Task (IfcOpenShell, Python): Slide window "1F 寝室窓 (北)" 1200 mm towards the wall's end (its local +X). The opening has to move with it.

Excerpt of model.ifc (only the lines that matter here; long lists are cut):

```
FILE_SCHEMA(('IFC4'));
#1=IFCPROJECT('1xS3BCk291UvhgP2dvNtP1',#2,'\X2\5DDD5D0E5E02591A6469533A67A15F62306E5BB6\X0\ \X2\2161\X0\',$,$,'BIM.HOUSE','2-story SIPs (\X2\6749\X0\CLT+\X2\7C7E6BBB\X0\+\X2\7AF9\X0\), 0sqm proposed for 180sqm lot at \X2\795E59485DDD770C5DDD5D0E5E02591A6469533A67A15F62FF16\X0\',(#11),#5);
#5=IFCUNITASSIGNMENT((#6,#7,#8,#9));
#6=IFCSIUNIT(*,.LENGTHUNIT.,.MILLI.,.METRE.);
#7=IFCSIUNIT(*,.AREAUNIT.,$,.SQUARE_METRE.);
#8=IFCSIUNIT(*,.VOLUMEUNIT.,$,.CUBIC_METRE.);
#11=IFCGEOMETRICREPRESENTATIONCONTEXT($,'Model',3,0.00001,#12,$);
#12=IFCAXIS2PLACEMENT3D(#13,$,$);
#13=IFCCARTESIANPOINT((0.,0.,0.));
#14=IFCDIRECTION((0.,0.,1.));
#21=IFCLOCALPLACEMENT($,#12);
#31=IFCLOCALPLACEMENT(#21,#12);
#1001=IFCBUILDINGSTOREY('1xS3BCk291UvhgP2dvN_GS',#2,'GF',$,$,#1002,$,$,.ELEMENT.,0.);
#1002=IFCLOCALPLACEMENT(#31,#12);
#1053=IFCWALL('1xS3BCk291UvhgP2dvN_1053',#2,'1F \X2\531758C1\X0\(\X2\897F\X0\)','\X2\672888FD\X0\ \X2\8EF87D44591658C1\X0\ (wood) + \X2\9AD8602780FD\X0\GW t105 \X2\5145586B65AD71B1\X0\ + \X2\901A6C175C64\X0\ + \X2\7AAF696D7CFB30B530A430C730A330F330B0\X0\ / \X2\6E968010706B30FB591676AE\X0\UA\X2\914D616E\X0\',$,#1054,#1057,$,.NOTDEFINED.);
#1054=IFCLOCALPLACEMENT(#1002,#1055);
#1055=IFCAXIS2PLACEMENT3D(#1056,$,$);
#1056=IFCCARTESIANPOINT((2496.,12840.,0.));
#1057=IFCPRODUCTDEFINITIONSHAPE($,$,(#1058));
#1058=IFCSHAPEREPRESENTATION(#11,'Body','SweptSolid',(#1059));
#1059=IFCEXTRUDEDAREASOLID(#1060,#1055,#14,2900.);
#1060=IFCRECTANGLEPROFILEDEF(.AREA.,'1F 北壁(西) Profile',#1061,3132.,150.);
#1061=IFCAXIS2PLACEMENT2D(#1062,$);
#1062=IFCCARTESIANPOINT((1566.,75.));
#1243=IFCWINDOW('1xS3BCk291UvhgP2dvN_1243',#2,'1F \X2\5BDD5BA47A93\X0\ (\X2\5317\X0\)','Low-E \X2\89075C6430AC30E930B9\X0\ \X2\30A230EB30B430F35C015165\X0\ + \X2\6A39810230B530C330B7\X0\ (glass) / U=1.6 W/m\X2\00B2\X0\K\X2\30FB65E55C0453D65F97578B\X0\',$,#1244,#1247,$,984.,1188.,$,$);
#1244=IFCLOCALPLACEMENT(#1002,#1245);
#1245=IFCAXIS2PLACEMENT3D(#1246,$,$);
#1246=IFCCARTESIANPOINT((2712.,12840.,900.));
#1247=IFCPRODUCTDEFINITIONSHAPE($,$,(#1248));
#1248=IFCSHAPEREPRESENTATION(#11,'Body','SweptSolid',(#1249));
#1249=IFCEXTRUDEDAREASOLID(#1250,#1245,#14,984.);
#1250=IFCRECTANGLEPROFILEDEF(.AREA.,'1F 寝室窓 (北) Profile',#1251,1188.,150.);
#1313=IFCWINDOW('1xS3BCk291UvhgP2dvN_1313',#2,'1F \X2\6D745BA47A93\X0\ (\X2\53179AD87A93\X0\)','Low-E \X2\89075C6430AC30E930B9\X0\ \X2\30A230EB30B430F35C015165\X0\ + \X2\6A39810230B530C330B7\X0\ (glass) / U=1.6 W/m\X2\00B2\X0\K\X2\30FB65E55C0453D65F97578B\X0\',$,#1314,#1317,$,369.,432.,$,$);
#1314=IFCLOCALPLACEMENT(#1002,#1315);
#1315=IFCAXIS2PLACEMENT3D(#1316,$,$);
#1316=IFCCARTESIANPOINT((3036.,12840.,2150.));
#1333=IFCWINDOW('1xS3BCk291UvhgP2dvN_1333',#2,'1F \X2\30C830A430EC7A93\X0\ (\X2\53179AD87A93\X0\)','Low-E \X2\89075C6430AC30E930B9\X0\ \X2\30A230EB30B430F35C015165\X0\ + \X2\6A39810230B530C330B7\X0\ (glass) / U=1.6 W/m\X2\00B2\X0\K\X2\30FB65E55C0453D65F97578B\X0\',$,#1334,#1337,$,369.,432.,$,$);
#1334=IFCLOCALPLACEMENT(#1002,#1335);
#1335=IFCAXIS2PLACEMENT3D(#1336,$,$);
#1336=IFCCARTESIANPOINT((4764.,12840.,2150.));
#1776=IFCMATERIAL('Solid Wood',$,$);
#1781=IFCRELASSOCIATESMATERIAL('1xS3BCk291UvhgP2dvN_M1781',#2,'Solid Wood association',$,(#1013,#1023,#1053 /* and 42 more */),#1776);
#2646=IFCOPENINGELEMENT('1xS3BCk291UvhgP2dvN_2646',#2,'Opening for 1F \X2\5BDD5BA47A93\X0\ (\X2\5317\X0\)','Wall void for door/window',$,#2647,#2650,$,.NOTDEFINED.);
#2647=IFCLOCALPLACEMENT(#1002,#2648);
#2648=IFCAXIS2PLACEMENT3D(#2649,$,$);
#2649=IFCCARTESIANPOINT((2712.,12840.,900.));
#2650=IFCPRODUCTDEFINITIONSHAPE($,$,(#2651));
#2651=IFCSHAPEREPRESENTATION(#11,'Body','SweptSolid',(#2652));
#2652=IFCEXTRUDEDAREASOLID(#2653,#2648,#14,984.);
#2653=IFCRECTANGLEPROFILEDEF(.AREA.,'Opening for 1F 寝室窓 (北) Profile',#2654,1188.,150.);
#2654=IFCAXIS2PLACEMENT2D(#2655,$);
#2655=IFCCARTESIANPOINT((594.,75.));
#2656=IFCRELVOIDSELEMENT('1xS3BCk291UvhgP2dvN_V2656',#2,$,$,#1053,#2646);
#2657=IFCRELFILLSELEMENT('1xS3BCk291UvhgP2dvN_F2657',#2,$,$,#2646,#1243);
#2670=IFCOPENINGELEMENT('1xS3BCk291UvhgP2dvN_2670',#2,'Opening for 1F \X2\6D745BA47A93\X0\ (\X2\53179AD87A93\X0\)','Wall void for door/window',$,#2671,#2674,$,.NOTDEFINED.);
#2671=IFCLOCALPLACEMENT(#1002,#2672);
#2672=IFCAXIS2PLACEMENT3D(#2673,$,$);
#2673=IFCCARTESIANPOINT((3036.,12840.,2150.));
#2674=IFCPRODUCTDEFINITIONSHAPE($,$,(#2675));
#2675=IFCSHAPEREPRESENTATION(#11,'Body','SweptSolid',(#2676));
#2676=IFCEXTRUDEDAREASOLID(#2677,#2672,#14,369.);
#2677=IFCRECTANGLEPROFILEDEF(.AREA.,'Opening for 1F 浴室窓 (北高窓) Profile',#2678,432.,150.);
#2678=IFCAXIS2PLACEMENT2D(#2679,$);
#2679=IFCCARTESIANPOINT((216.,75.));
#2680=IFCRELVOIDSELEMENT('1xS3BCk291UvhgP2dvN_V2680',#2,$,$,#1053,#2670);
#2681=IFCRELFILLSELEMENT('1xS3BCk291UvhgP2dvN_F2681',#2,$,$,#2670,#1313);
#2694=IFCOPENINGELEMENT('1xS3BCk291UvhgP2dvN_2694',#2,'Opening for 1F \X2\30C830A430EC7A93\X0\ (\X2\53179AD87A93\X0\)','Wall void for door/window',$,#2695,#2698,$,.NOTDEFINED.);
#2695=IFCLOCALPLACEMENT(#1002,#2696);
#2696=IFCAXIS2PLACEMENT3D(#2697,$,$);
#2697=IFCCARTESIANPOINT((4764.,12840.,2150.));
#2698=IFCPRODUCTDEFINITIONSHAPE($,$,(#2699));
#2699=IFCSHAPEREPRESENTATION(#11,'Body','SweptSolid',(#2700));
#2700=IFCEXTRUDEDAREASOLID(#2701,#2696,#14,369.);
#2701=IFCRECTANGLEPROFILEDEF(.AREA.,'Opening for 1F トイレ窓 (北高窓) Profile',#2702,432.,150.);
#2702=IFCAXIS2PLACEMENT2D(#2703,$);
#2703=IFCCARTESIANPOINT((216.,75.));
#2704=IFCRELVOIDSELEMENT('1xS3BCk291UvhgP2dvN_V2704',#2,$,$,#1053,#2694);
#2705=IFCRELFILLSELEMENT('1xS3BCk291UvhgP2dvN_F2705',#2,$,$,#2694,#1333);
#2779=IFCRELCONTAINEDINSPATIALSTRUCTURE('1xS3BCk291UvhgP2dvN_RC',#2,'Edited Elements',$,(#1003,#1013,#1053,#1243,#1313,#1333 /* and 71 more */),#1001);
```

```python
import ifcopenshell
import ifcopenshell.api.geometry
import ifcopenshell.util.placement

model = ifcopenshell.open("model.ifc")

window = model.by_guid("1xS3BCk291UvhgP2dvN_1243")
opening = window.FillsVoids[0].RelatingOpeningElement
wall = opening.VoidsElements[0].RelatingBuildingElement

wall_matrix = ifcopenshell.util.placement.get_local_placement(wall.ObjectPlacement)
shift = wall_matrix[:3, 0] * 1200.0
before = ifcopenshell.util.placement.get_local_placement(window.ObjectPlacement)[:3, 3].copy()

# The window is not placed relative to its opening, so move both.
for product in (opening, window):
    matrix = ifcopenshell.util.placement.get_local_placement(product.ObjectPlacement)
    matrix[:3, 3] += shift
    ifcopenshell.api.geometry.edit_object_placement(model, product=product, matrix=matrix, is_si=False)

after = ifcopenshell.util.placement.get_local_placement(window.ObjectPlacement)[:3, 3]
print("window moved by", (after - before).round(3) + 0.0)

model.write("model-out.ifc")
```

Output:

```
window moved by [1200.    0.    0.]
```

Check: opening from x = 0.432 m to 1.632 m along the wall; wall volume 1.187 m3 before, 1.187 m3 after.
